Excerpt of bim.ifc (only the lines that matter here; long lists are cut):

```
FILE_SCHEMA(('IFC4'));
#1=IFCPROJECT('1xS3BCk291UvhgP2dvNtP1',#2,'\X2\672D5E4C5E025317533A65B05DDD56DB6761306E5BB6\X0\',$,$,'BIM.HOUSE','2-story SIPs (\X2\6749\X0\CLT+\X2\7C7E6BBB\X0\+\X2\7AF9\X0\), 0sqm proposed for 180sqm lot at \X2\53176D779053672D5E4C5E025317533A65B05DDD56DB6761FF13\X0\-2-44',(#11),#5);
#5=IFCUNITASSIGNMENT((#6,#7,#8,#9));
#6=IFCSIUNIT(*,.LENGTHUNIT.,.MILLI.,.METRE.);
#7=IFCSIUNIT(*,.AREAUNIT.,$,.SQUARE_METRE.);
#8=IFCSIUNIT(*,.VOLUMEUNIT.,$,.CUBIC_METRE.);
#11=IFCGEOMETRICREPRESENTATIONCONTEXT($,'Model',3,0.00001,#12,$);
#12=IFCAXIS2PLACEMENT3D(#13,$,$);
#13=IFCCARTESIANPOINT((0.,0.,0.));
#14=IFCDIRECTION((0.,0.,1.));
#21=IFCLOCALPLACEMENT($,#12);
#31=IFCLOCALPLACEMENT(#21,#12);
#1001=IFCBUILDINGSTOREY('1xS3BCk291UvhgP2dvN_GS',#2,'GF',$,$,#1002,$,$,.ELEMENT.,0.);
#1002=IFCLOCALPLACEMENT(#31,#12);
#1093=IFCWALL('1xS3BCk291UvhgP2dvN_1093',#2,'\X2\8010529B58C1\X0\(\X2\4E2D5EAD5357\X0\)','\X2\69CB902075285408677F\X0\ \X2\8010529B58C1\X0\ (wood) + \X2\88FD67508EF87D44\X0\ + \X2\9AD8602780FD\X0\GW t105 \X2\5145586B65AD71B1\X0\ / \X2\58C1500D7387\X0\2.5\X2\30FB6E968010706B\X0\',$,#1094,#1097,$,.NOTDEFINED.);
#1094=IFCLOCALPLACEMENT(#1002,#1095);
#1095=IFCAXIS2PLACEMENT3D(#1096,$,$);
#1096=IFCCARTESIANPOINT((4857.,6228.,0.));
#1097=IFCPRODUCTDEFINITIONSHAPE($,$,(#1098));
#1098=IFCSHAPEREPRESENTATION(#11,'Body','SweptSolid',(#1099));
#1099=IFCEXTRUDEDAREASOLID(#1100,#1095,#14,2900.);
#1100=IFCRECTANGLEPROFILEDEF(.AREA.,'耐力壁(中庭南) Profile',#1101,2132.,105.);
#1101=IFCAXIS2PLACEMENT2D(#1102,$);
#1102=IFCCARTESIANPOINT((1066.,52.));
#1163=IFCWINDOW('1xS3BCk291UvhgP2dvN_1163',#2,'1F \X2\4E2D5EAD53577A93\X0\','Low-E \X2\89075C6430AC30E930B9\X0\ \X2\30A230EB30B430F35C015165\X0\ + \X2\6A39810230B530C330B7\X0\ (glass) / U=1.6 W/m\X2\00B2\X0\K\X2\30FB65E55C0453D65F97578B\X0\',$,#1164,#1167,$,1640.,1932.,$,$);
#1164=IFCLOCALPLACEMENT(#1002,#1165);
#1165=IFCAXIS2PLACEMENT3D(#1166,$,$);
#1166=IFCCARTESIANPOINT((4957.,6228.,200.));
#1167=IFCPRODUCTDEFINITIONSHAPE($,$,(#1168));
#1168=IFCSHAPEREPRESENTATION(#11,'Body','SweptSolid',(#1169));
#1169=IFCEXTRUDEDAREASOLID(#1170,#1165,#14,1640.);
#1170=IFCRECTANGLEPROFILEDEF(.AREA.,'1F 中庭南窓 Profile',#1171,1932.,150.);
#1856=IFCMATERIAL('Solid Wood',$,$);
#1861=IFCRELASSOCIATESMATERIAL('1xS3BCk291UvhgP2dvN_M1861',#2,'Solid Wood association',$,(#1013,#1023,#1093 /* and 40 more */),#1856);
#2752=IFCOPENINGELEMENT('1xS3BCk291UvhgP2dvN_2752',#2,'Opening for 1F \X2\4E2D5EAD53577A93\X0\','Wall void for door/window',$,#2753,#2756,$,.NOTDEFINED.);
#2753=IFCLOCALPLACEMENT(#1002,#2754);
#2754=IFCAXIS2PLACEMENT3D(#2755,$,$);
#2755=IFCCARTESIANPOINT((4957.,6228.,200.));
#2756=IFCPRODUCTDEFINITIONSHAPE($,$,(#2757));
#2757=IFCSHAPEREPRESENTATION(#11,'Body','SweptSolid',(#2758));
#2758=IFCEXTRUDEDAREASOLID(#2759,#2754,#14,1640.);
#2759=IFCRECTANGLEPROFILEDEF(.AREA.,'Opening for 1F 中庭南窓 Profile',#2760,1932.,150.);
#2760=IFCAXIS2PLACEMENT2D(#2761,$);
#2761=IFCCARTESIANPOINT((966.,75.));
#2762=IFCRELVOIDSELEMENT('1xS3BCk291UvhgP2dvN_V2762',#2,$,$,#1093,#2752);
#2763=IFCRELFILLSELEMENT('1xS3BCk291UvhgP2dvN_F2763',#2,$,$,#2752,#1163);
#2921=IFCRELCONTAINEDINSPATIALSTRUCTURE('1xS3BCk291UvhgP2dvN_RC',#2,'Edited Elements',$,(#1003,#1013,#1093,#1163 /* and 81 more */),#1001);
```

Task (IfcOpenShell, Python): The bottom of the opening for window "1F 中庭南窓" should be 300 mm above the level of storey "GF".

```python
import numpy as np
import ifcopenshell
import ifcopenshell.api.geometry
import ifcopenshell.geom
import ifcopenshell.util.element
import ifcopenshell.util.placement
import ifcopenshell.util.shape
import ifcopenshell.util.unit

model = ifcopenshell.open("bim.ifc")
unit_scale = ifcopenshell.util.unit.calculate_unit_scale(model)

window = model.by_guid("1xS3BCk291UvhgP2dvN_1163")
opening = window.FillsVoids[0].RelatingOpeningElement
storey = ifcopenshell.util.element.get_container(window, ifc_class="IfcBuildingStorey")
level = ifcopenshell.util.placement.get_local_placement(storey.ObjectPlacement)[2, 3]

# The opening's origin need not be at the sill, so measure its lowest point.
shape = ifcopenshell.geom.create_shape(ifcopenshell.geom.settings(), opening)
bottom = ifcopenshell.util.shape.get_shape_bottom_elevation(shape, shape.geometry) / unit_scale
dz = level + 0.3 / unit_scale - bottom

shift = np.array([0.0, 0.0, dz])
# The window is not placed relative to its opening, so move both.
for product in (opening, window):
    matrix = ifcopenshell.util.placement.get_local_placement(product.ObjectPlacement)
    matrix[:3, 3] += shift
    ifcopenshell.api.geometry.edit_object_placement(model, product=product, matrix=matrix, is_si=False)

print(f"moved by {dz * unit_scale:+.3f} m")

model.write("bim_v2.ifc")
```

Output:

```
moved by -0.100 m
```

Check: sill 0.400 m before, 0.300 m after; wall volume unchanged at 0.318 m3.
